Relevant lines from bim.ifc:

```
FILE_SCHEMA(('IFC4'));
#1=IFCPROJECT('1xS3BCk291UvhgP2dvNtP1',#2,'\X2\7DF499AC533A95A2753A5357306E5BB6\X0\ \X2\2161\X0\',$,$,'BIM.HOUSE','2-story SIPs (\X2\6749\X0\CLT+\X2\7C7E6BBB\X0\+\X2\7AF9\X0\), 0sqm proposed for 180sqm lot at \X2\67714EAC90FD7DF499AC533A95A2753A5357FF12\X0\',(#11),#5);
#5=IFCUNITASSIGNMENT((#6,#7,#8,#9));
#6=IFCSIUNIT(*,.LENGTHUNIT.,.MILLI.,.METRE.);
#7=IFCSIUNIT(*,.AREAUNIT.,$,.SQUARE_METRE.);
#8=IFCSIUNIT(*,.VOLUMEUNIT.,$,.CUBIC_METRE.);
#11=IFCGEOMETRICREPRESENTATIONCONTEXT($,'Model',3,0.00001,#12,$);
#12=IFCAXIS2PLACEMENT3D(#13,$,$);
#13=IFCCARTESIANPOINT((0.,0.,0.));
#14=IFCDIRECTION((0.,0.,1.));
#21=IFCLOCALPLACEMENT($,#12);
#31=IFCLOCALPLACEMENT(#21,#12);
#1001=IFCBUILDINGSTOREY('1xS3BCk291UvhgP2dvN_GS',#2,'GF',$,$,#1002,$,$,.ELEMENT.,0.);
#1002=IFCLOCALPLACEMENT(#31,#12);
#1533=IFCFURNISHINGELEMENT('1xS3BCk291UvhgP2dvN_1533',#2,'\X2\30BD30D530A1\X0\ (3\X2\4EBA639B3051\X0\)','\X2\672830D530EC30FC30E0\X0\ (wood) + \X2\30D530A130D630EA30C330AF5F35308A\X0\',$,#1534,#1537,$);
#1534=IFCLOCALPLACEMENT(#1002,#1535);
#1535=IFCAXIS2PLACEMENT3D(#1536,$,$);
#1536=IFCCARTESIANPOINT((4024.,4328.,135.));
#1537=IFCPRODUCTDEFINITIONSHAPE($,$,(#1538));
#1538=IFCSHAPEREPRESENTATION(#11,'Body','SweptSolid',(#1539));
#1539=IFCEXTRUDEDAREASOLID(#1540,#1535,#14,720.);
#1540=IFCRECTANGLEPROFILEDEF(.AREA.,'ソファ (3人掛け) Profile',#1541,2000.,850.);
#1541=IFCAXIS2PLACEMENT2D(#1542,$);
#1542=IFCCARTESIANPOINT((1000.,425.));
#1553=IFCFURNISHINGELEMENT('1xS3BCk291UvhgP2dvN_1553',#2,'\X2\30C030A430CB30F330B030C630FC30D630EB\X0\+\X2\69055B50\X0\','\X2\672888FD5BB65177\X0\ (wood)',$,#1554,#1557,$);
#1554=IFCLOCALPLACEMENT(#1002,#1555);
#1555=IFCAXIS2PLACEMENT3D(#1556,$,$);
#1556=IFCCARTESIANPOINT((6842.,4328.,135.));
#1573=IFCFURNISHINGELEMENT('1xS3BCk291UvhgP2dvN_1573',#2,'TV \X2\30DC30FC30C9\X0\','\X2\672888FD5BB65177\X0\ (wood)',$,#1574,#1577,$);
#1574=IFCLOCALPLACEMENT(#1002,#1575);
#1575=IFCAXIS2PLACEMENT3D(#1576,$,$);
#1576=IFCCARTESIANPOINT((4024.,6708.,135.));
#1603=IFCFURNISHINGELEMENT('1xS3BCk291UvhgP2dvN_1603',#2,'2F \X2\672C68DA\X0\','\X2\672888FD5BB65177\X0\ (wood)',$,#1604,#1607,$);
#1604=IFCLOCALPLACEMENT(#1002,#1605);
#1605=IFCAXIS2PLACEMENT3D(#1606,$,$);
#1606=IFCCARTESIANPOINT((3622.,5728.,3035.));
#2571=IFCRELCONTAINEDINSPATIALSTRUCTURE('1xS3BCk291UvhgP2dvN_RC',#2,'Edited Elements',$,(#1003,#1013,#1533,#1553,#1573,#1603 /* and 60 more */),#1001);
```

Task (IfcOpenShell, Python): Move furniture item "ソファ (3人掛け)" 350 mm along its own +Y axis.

```python
import ifcopenshell
import ifcopenshell.api.geometry
import ifcopenshell.util.placement
import ifcopenshell.util.unit

model = ifcopenshell.open("bim.ifc")
unit_scale = ifcopenshell.util.unit.calculate_unit_scale(model)

item = model.by_guid("1xS3BCk291UvhgP2dvN_1533")
matrix = ifcopenshell.util.placement.get_local_placement(item.ObjectPlacement)
matrix[:3, 3] += matrix[:3, 1] * 0.35 / unit_scale
ifcopenshell.api.geometry.edit_object_placement(model, product=item, matrix=matrix, is_si=False)

print(ifcopenshell.util.placement.get_local_placement(item.ObjectPlacement).round(3) + 0.0)

model.write("bim-out.ifc")
```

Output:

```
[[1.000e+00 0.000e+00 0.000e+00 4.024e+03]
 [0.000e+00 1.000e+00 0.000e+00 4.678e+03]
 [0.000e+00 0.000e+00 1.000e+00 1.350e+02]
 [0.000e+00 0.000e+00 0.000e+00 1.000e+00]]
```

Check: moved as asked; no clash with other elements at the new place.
